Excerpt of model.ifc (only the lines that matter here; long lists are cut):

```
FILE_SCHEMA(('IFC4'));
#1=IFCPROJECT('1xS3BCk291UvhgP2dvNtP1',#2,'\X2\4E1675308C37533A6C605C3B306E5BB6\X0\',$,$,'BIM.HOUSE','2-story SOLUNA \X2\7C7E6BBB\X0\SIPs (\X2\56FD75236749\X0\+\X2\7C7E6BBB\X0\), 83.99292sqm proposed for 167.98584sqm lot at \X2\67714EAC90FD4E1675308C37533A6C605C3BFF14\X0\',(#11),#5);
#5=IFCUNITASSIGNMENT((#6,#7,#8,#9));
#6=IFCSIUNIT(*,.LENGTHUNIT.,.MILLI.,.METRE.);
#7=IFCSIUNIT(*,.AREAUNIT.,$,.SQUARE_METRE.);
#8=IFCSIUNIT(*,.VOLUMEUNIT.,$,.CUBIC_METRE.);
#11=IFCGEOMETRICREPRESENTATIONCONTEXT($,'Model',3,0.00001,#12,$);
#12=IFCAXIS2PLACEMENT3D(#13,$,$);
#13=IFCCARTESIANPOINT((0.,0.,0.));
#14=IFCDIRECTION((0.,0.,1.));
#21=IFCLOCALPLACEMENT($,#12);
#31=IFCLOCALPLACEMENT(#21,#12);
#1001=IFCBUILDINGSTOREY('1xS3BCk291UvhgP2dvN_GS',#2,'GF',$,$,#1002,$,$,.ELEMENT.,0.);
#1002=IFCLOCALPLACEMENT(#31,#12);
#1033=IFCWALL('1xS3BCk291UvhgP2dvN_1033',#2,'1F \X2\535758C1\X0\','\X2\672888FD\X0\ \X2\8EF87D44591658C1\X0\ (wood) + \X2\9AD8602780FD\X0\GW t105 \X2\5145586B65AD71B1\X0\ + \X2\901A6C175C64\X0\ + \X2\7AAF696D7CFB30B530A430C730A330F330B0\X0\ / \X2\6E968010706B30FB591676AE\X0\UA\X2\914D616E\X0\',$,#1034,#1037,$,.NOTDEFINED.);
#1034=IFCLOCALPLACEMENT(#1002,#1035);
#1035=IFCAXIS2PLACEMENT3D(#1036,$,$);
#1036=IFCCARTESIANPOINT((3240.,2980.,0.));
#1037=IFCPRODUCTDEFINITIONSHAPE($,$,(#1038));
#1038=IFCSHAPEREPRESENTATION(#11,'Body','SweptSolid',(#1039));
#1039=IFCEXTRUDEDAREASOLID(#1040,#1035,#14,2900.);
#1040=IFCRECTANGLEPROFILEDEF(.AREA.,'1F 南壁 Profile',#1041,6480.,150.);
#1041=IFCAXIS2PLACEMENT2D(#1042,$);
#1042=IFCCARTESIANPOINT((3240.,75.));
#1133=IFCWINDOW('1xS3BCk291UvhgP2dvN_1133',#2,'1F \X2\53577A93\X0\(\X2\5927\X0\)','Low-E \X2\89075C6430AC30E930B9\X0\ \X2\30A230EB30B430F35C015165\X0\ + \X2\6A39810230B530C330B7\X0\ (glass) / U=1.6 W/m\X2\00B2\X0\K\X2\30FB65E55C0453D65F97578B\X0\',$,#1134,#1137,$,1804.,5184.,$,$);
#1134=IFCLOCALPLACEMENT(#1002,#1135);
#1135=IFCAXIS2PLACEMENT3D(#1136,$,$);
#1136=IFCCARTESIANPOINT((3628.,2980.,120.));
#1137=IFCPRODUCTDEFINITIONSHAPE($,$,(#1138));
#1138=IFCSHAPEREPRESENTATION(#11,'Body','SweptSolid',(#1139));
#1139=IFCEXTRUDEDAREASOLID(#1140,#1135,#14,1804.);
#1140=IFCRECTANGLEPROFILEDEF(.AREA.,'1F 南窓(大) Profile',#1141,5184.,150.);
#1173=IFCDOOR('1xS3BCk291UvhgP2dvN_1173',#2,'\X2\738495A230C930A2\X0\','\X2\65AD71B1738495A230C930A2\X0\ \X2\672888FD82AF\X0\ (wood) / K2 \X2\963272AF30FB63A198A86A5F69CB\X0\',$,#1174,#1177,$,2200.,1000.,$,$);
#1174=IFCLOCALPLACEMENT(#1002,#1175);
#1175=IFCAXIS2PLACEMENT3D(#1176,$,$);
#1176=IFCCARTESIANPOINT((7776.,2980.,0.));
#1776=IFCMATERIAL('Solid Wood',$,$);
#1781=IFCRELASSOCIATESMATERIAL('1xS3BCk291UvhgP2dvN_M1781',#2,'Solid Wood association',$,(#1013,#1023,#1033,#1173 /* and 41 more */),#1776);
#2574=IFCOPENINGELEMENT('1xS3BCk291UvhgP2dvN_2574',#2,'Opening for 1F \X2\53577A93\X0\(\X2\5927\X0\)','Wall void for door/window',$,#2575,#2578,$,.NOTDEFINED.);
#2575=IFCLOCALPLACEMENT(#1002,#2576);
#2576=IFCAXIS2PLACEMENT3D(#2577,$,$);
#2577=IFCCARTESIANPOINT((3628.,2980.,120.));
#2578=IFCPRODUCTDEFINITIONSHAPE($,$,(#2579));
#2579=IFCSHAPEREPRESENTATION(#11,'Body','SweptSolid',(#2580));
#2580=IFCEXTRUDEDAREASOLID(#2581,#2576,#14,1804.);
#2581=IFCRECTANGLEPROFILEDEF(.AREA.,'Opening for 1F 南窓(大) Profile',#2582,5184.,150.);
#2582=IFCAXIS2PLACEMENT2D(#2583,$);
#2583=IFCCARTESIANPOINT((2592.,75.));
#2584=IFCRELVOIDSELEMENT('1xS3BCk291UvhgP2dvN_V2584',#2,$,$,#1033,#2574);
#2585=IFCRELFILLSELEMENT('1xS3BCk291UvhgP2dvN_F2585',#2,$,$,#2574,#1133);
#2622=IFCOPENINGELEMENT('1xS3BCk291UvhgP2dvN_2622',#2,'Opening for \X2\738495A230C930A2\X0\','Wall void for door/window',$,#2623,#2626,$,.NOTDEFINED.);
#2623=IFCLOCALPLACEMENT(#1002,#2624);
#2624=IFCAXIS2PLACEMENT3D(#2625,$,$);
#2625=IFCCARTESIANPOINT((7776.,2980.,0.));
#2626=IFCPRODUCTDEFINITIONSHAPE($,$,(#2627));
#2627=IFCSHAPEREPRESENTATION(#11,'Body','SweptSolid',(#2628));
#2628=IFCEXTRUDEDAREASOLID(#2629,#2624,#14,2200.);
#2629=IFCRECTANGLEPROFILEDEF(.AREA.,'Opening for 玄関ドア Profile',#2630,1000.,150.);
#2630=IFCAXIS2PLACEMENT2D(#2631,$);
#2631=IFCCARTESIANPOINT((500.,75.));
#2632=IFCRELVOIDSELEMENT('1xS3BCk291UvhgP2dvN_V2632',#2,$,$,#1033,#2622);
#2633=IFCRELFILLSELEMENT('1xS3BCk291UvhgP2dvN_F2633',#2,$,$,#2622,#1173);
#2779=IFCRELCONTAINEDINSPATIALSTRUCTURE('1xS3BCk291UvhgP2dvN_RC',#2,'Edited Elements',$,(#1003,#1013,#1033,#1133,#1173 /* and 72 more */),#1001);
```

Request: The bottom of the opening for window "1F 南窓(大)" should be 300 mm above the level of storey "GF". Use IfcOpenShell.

```python
import numpy as np
import ifcopenshell
import ifcopenshell.api.geometry
import ifcopenshell.geom
import ifcopenshell.util.element
import ifcopenshell.util.placement
import ifcopenshell.util.shape
import ifcopenshell.util.unit

model = ifcopenshell.open("model.ifc")
unit_scale = ifcopenshell.util.unit.calculate_unit_scale(model)

window = model.by_guid("1xS3BCk291UvhgP2dvN_1133")
opening = window.FillsVoids[0].RelatingOpeningElement
storey = ifcopenshell.util.element.get_container(window, ifc_class="IfcBuildingStorey")
level = ifcopenshell.util.placement.get_local_placement(storey.ObjectPlacement)[2, 3]

# The opening's origin need not be at the sill, so measure its lowest point.
shape = ifcopenshell.geom.create_shape(ifcopenshell.geom.settings(), opening)
bottom = ifcopenshell.util.shape.get_shape_bottom_elevation(shape, shape.geometry) / unit_scale
dz = level + 0.3 / unit_scale - bottom

shift = np.array([0.0, 0.0, dz])
# The window is not placed relative to its opening, so move both.
for product in (opening, window):
    matrix = ifcopenshell.util.placement.get_local_placement(product.ObjectPlacement)
    matrix[:3, 3] += shift
    ifcopenshell.api.geometry.edit_object_placement(model, product=product, matrix=matrix, is_si=False)

print(f"moved by {dz * unit_scale:+.3f} m")

model.write("model_updated.ifc")
```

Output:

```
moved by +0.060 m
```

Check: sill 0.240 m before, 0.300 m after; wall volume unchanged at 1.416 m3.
